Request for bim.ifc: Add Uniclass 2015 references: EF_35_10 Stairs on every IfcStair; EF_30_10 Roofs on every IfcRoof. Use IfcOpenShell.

First a look at what the model holds.

```python
import ifcopenshell

model = ifcopenshell.open("bim.ifc")
print(model.schema)
print("classifications:", [c.Name for c in model.by_type("IfcClassification")])
for ifc_class in ("IfcDoor", "IfcRoof", "IfcStair", "IfcWall", "IfcWindow"):
    print(ifc_class, len(model.by_type(ifc_class)))
```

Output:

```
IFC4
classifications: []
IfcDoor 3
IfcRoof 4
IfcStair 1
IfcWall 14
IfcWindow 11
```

```python
import ifcopenshell
import ifcopenshell.api.classification

model = ifcopenshell.open("bim.ifc")

system = ifcopenshell.api.classification.add_classification(model, classification="Uniclass 2015")

codes = {
    "IfcStair": ("EF_35_10", "Stairs"),
    "IfcRoof": ("EF_30_10", "Roofs"),
}
for ifc_class, (code, name) in codes.items():
    products = model.by_type(ifc_class)
    ifcopenshell.api.classification.add_reference(
        model, products=products, classification=system, identification=code, name=name
    )
    print(code, len(products))

model.write("bim_v2.ifc")
```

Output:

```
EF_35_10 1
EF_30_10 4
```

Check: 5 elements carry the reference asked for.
